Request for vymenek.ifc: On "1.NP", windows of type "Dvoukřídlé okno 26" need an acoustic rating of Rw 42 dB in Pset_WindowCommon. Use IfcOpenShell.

First a look at what the model holds.

```python
import ifcopenshell
import ifcopenshell.util.element

model = ifcopenshell.open("vymenek.ifc")
print(model.schema)
storey = next(s for s in model.by_type("IfcBuildingStorey") if s.Name == "1.NP")
windows = [e for e in ifcopenshell.util.element.get_decomposition(storey) if e.is_a("IfcWindow")]
seen = {}
for e in windows:
    element_type = ifcopenshell.util.element.get_type(e)
    key = (element_type.Name if element_type != e and element_type else None, ifcopenshell.util.element.get_pset(e, "Pset_WindowCommon", "AcousticRating"))
    seen[key] = seen.get(key, 0) + 1
for (name, value), count in sorted(seen.items(), key=str):
    print(count, "x", name, "|", value)
```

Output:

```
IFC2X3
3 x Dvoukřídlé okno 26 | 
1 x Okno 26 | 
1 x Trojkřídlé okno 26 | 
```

```python
import ifcopenshell
import ifcopenshell.api.pset
import ifcopenshell.util.element

model = ifcopenshell.open("vymenek.ifc")

storey = next(s for s in model.by_type("IfcBuildingStorey") if s.Name == "1.NP")
windows = [e for e in ifcopenshell.util.element.get_decomposition(storey) if e.is_a("IfcWindow")]

count = 0
for e in windows:
    element_type = ifcopenshell.util.element.get_type(e)
    if element_type in (None, e) or element_type.Name != "Dvoukřídlé okno 26":
        continue
    # add_pset returns the element's existing set when there is one.
    pset = ifcopenshell.api.pset.add_pset(model, product=e, name="Pset_WindowCommon")
    ifcopenshell.api.pset.edit_pset(model, pset=pset, properties={"AcousticRating": "Rw 42 dB"})
    count += 1

print(count, "windows updated")

model.write("vymenek-out.ifc")
```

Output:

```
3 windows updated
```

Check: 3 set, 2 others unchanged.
